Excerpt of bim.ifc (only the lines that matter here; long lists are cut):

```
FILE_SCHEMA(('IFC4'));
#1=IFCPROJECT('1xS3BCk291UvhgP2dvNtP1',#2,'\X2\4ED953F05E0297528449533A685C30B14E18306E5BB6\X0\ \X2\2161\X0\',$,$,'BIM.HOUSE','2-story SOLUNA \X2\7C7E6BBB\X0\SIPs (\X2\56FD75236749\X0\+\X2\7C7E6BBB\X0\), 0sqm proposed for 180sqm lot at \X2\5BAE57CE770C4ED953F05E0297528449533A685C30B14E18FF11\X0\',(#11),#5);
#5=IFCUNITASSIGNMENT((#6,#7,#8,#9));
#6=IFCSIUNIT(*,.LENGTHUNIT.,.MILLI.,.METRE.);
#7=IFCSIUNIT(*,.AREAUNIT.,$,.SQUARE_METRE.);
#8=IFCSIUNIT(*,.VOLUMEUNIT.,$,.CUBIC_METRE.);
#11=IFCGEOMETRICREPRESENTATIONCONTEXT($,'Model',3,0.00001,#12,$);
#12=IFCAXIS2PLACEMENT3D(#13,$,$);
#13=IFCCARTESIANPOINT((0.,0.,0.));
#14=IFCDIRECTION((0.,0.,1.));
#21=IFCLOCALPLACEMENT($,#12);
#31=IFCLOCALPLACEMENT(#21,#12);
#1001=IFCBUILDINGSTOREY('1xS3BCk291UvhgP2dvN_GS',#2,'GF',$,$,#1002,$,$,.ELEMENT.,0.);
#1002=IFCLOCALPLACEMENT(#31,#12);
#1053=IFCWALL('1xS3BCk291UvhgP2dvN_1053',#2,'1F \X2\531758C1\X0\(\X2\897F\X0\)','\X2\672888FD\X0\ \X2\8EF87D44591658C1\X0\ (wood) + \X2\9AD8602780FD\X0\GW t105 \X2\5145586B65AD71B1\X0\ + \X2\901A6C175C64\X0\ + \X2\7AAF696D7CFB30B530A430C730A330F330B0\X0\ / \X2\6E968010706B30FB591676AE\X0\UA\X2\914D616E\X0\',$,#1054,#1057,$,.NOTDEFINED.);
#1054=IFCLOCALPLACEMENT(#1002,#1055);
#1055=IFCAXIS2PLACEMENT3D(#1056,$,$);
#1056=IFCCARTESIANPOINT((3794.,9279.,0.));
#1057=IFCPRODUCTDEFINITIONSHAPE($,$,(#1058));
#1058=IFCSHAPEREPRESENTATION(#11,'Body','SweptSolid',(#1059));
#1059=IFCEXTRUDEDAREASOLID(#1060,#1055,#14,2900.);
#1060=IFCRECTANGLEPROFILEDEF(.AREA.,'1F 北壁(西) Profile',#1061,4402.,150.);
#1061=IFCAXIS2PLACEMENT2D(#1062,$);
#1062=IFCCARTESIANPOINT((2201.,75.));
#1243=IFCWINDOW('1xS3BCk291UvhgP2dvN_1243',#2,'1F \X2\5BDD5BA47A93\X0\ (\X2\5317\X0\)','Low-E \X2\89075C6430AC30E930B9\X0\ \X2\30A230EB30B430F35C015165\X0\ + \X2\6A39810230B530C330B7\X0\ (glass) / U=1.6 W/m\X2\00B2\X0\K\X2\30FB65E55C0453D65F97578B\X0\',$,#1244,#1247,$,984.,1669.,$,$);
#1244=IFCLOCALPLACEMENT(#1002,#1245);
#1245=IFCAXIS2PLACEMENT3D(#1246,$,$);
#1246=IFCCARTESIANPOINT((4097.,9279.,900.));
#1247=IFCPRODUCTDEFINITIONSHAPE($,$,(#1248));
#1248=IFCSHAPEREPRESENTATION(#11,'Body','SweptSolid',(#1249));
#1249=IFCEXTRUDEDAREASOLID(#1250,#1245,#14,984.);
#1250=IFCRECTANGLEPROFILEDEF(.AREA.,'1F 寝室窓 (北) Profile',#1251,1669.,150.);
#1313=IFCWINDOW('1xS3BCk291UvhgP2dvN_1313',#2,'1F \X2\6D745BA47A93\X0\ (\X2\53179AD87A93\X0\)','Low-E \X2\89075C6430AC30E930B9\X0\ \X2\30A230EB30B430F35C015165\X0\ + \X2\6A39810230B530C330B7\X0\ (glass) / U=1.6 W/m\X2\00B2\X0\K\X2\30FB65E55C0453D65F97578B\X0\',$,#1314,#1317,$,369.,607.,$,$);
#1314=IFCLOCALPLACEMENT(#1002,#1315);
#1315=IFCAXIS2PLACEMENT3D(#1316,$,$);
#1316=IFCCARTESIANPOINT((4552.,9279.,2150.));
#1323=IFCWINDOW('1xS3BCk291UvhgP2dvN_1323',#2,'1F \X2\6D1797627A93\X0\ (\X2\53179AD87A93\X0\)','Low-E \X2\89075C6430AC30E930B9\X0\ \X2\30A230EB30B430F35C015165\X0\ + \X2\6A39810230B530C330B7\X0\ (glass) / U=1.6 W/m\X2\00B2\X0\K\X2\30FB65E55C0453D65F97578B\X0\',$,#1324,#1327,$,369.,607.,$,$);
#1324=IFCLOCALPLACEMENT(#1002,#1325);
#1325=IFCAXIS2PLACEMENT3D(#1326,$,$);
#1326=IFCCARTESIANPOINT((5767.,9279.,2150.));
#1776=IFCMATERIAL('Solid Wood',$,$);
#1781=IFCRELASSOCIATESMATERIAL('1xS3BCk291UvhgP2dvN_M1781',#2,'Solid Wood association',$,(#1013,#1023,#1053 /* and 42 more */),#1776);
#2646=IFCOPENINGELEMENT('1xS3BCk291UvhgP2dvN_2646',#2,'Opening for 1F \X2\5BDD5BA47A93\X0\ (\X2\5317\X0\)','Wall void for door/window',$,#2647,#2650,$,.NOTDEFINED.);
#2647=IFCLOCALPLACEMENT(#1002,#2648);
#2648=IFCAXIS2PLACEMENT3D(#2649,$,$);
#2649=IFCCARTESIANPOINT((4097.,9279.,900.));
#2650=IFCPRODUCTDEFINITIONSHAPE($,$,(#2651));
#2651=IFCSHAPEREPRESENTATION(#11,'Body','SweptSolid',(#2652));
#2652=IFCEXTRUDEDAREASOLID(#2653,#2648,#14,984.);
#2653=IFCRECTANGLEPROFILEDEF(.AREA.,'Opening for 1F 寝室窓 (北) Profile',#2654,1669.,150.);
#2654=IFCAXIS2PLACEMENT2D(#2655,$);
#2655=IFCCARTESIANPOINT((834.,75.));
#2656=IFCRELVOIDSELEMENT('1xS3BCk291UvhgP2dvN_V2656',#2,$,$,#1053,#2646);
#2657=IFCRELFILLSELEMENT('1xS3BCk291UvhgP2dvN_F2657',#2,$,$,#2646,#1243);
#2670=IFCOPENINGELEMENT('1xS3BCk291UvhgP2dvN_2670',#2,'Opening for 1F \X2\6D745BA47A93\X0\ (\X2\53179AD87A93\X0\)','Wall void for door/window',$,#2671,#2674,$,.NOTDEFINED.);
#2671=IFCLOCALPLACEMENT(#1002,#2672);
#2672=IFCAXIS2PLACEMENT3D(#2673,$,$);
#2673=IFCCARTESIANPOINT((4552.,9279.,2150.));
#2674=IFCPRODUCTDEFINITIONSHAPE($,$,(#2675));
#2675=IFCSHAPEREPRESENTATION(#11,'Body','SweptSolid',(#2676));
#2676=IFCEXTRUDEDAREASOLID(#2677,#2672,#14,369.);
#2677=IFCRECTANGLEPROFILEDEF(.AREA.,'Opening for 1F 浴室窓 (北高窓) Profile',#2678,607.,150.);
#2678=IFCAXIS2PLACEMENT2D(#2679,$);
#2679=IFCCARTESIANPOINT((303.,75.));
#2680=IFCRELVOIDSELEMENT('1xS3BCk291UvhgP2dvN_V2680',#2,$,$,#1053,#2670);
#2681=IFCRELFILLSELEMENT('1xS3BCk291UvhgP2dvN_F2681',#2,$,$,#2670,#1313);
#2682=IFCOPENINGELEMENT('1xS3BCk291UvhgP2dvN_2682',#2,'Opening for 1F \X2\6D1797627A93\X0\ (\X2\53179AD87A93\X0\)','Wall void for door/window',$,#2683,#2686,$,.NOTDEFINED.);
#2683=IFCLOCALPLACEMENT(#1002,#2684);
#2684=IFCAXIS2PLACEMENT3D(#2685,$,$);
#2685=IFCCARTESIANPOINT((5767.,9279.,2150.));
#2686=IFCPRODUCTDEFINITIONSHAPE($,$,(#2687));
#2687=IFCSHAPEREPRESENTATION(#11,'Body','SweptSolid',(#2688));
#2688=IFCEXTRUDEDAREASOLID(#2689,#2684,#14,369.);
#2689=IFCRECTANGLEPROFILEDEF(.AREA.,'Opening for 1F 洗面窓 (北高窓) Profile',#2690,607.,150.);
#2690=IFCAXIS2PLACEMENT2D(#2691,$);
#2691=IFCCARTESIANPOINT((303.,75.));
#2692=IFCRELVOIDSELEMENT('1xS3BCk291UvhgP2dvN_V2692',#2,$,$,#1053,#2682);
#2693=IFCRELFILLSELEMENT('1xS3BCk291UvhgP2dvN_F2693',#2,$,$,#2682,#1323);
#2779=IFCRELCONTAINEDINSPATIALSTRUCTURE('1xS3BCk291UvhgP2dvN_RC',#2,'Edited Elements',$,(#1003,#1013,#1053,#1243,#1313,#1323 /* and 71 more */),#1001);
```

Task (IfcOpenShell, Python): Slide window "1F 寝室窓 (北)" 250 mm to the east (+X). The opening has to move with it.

```python
import ifcopenshell
import ifcopenshell.api.geometry
import ifcopenshell.util.placement

model = ifcopenshell.open("bim.ifc")

window = model.by_guid("1xS3BCk291UvhgP2dvN_1243")
opening = window.FillsVoids[0].RelatingOpeningElement
wall = opening.VoidsElements[0].RelatingBuildingElement

wall_matrix = ifcopenshell.util.placement.get_local_placement(wall.ObjectPlacement)
shift = wall_matrix[:3, 0] * 250.0
before = ifcopenshell.util.placement.get_local_placement(window.ObjectPlacement)[:3, 3].copy()

# The window is not placed relative to its opening, so move both.
for product in (opening, window):
    matrix = ifcopenshell.util.placement.get_local_placement(product.ObjectPlacement)
    matrix[:3, 3] += shift
    ifcopenshell.api.geometry.edit_object_placement(model, product=product, matrix=matrix, is_si=False)

after = ifcopenshell.util.placement.get_local_placement(window.ObjectPlacement)[:3, 3]
print("window moved by", (after - before).round(3) + 0.0)

model.write("bim-out.ifc")
```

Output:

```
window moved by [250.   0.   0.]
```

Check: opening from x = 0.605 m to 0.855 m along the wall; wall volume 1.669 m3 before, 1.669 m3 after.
